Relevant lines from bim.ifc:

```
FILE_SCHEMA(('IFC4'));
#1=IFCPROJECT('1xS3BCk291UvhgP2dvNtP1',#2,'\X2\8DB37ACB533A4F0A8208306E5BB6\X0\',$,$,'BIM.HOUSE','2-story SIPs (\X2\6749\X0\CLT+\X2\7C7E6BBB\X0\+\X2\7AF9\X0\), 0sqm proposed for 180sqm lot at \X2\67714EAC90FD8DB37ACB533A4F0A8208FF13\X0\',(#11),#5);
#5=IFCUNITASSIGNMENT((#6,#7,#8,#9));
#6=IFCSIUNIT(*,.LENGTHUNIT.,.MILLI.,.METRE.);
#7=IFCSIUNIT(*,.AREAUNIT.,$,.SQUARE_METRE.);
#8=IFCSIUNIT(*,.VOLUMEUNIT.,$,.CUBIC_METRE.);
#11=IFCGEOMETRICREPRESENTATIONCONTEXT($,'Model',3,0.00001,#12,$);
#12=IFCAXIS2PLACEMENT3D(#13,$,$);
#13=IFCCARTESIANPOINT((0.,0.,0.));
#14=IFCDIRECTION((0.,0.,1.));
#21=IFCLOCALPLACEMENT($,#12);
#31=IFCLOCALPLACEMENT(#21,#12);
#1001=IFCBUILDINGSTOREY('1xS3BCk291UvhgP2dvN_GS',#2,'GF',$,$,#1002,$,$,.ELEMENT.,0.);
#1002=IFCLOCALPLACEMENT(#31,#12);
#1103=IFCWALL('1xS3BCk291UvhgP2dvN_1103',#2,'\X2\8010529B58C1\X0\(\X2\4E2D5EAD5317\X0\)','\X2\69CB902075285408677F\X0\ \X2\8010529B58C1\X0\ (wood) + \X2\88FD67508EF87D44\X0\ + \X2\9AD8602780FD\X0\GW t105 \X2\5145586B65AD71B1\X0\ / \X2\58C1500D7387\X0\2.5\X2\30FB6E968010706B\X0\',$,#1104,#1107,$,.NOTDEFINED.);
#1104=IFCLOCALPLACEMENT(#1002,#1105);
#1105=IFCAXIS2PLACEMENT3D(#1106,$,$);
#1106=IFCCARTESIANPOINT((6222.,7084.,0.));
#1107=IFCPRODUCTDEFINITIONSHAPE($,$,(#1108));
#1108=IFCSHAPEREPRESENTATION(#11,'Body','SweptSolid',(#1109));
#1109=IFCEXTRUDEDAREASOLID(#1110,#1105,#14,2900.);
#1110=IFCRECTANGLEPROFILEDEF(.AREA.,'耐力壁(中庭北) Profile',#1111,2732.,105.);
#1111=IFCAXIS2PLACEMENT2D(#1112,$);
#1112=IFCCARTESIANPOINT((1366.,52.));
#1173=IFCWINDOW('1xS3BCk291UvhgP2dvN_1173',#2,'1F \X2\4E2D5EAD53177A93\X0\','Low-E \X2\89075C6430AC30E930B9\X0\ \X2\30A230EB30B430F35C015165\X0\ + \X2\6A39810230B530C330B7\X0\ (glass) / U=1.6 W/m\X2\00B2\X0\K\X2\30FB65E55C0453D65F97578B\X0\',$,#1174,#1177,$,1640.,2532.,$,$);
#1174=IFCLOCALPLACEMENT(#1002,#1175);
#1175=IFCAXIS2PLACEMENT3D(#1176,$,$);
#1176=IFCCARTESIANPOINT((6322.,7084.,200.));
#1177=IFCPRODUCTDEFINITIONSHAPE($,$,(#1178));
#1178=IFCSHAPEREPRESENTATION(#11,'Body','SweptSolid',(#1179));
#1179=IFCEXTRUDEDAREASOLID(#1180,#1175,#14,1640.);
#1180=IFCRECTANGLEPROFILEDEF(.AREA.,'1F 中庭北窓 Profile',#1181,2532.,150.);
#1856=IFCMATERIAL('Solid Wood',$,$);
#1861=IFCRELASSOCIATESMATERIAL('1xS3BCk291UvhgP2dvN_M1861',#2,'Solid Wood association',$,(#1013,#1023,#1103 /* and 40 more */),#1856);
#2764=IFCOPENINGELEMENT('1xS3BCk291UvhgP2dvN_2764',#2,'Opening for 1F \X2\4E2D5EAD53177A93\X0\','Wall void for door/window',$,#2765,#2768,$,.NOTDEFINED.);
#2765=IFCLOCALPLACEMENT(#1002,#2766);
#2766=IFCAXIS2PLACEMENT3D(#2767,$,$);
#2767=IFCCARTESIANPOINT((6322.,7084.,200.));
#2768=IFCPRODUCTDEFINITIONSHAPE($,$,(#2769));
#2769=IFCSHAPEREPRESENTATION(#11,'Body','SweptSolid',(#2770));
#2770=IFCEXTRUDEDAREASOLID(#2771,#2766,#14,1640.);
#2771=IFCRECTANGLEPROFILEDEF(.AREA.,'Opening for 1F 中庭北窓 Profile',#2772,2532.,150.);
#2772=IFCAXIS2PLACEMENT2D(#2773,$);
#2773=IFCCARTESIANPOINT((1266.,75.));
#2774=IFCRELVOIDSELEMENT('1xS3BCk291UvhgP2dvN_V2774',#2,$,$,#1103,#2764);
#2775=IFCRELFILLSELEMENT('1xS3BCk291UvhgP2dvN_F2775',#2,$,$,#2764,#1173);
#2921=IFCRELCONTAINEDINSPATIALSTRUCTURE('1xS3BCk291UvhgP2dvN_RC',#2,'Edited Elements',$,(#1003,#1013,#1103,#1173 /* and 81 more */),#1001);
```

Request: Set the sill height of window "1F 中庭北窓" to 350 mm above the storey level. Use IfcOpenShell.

```python
import numpy as np
import ifcopenshell
import ifcopenshell.api.geometry
import ifcopenshell.geom
import ifcopenshell.util.element
import ifcopenshell.util.placement
import ifcopenshell.util.shape
import ifcopenshell.util.unit

model = ifcopenshell.open("bim.ifc")
unit_scale = ifcopenshell.util.unit.calculate_unit_scale(model)

window = model.by_guid("1xS3BCk291UvhgP2dvN_1173")
opening = window.FillsVoids[0].RelatingOpeningElement
storey = ifcopenshell.util.element.get_container(window, ifc_class="IfcBuildingStorey")
level = ifcopenshell.util.placement.get_local_placement(storey.ObjectPlacement)[2, 3]

# The opening's origin need not be at the sill, so measure its lowest point.
shape = ifcopenshell.geom.create_shape(ifcopenshell.geom.settings(), opening)
bottom = ifcopenshell.util.shape.get_shape_bottom_elevation(shape, shape.geometry) / unit_scale
dz = level + 0.35 / unit_scale - bottom

shift = np.array([0.0, 0.0, dz])
# The window is not placed relative to its opening, so move both.
for product in (opening, window):
    matrix = ifcopenshell.util.placement.get_local_placement(product.ObjectPlacement)
    matrix[:3, 3] += shift
    ifcopenshell.api.geometry.edit_object_placement(model, product=product, matrix=matrix, is_si=False)

print(f"moved by {dz * unit_scale:+.3f} m")

model.write("bim_updated.ifc")
```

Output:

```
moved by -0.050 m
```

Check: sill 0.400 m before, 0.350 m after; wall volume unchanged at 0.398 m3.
